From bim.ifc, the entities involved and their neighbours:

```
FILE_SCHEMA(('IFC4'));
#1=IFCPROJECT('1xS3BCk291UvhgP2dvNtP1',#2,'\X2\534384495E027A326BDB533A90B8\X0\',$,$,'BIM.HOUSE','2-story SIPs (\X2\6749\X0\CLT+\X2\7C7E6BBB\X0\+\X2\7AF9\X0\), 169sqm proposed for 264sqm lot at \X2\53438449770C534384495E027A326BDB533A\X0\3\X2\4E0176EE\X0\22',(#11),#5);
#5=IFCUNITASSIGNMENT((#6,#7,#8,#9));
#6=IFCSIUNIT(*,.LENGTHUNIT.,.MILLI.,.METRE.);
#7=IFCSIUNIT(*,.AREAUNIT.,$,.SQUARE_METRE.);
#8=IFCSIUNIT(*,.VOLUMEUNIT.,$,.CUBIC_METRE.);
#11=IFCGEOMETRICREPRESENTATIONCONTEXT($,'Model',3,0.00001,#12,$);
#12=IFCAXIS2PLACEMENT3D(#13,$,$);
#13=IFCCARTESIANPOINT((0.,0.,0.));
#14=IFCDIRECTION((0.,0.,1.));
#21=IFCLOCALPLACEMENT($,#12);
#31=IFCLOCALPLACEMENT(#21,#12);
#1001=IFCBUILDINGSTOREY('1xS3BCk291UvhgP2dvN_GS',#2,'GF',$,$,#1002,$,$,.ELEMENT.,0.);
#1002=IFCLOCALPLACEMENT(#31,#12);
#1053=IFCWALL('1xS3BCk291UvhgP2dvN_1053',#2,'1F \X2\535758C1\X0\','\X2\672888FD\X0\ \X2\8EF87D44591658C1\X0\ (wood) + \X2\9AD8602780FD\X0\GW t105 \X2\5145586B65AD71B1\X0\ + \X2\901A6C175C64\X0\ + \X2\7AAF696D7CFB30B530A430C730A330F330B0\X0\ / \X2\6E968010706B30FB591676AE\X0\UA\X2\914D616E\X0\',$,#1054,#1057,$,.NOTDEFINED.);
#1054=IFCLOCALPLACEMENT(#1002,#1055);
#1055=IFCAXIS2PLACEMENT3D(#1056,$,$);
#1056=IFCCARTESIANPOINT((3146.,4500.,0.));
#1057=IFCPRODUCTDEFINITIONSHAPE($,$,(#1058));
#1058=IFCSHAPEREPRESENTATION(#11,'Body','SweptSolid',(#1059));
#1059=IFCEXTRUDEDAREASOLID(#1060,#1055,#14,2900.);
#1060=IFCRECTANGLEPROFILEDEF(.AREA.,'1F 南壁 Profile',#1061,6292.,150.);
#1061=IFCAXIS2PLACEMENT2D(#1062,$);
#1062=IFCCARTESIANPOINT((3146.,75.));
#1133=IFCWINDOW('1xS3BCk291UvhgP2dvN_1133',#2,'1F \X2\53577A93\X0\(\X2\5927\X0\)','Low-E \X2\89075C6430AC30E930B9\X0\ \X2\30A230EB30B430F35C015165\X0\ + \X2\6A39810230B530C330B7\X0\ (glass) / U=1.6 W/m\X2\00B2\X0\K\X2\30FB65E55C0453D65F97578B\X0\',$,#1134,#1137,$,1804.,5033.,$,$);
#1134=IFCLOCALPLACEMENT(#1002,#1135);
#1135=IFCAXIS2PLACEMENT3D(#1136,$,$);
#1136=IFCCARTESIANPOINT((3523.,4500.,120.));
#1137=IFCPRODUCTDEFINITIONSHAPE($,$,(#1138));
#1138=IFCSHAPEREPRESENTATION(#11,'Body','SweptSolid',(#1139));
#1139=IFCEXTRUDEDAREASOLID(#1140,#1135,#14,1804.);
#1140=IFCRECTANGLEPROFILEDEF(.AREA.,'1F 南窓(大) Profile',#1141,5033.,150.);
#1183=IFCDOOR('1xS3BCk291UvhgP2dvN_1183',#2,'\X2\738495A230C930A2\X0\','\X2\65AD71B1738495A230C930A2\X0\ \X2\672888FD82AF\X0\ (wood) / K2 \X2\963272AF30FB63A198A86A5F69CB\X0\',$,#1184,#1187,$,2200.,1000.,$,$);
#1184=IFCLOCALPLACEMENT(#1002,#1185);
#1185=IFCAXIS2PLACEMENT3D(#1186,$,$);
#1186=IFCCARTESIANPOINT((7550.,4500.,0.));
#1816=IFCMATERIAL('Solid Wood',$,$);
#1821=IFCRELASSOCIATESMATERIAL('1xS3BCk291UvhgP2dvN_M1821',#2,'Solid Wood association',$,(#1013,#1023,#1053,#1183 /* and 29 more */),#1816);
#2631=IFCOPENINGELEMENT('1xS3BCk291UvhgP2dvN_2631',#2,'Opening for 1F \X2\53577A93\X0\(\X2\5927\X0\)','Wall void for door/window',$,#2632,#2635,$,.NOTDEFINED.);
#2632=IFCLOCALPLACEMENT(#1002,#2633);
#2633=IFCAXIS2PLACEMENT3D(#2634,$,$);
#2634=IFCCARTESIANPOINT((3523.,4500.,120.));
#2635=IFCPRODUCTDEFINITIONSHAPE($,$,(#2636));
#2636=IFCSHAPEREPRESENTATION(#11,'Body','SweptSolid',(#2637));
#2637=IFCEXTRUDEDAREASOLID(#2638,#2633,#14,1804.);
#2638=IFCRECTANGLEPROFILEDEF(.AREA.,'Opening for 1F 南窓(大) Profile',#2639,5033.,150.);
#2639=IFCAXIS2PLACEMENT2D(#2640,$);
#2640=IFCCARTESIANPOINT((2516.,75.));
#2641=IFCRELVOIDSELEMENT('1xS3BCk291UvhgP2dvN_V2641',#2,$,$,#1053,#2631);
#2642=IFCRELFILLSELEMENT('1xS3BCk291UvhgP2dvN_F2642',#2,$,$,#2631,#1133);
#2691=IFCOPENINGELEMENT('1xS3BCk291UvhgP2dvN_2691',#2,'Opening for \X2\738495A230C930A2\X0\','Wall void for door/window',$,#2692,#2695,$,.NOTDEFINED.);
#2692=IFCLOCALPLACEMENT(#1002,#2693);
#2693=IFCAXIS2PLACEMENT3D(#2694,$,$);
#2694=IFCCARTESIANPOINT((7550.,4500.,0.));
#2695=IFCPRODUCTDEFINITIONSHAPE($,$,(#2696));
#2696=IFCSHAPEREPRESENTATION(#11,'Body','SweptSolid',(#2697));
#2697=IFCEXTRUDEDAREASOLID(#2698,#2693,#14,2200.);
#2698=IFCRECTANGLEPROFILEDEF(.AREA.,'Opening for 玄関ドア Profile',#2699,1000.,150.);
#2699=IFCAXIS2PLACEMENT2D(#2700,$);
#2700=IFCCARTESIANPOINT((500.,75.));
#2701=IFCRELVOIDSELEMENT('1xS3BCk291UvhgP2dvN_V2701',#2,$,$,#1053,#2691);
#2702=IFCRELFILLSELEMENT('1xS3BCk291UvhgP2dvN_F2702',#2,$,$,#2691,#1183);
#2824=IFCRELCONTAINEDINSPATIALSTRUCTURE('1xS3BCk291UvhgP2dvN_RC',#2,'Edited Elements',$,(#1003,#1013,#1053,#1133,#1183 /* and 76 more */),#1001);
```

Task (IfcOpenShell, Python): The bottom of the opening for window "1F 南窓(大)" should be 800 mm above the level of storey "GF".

```python
import numpy as np
import ifcopenshell
import ifcopenshell.api.geometry
import ifcopenshell.geom
import ifcopenshell.util.element
import ifcopenshell.util.placement
import ifcopenshell.util.shape
import ifcopenshell.util.unit

model = ifcopenshell.open("bim.ifc")
unit_scale = ifcopenshell.util.unit.calculate_unit_scale(model)

window = model.by_id(1133)
opening = window.FillsVoids[0].RelatingOpeningElement
storey = ifcopenshell.util.element.get_container(window, ifc_class="IfcBuildingStorey")
level = ifcopenshell.util.placement.get_local_placement(storey.ObjectPlacement)[2, 3]

# The opening's origin need not be at the sill, so measure its lowest point.
shape = ifcopenshell.geom.create_shape(ifcopenshell.geom.settings(), opening)
bottom = ifcopenshell.util.shape.get_shape_bottom_elevation(shape, shape.geometry) / unit_scale
dz = level + 0.8 / unit_scale - bottom

shift = np.array([0.0, 0.0, dz])
# The window is not placed relative to its opening, so move both.
for product in (opening, window):
    matrix = ifcopenshell.util.placement.get_local_placement(product.ObjectPlacement)
    matrix[:3, 3] += shift
    ifcopenshell.api.geometry.edit_object_placement(model, product=product, matrix=matrix, is_si=False)

print(f"moved by {dz * unit_scale:+.3f} m")

model.write("bim-out.ifc")
```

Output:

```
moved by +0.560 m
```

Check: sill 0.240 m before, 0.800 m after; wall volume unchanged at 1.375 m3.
